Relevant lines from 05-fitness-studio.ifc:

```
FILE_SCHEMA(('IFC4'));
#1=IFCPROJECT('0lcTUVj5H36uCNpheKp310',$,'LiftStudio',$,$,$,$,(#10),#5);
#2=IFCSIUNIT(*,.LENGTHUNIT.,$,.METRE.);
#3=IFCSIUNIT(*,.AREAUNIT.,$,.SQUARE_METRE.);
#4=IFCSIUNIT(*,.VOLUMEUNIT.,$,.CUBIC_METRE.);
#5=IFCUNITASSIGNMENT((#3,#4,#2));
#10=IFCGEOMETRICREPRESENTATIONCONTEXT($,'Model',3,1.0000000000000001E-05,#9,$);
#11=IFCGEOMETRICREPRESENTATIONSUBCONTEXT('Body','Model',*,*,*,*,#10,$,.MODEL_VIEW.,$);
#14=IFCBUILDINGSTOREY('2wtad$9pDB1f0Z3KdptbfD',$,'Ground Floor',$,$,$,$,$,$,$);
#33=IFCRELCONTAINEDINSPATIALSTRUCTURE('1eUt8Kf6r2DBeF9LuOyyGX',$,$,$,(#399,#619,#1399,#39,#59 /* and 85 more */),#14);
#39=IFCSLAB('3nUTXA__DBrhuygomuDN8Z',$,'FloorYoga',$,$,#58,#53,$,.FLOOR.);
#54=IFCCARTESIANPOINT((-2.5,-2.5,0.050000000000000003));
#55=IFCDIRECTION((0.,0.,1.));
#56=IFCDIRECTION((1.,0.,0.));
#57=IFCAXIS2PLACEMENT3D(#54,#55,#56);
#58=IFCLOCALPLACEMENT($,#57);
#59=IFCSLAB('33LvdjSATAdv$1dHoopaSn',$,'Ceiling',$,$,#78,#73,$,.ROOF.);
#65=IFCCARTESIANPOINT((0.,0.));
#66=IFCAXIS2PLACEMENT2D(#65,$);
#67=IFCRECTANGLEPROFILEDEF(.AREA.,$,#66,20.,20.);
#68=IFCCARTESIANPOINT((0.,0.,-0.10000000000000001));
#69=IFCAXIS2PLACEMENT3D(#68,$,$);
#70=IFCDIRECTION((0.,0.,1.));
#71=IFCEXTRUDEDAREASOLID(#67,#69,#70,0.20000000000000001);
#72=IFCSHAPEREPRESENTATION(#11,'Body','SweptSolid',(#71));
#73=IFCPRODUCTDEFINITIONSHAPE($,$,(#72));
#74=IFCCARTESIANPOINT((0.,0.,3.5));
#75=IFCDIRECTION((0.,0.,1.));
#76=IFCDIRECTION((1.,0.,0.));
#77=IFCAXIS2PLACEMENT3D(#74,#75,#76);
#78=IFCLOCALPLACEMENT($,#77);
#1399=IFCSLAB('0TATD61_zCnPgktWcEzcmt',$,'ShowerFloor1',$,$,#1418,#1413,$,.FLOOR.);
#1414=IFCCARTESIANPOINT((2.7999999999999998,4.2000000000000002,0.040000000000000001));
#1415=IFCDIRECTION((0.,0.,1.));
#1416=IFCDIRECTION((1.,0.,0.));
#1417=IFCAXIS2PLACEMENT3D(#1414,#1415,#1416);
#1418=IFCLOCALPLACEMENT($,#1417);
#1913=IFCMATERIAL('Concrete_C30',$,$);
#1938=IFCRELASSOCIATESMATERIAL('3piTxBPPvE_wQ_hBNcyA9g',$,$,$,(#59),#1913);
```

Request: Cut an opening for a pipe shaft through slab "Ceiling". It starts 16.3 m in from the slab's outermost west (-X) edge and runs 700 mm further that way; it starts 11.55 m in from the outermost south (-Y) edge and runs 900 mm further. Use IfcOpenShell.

```python
import numpy as np
import ifcopenshell
import ifcopenshell.api.feature
import ifcopenshell.api.geometry
import ifcopenshell.api.root
import ifcopenshell.geom
import ifcopenshell.util.placement
import ifcopenshell.util.representation
import ifcopenshell.util.shape
import ifcopenshell.util.unit

model = ifcopenshell.open("05-fitness-studio.ifc")
unit_scale = ifcopenshell.util.unit.calculate_unit_scale(model)
settings = ifcopenshell.geom.settings()


def volume(element):
    """Net volume in cubic metres, openings subtracted."""
    shape = ifcopenshell.geom.create_shape(settings, element)
    return ifcopenshell.util.shape.get_volume(shape.geometry)


slab = model.by_guid("33LvdjSATAdv$1dHoopaSn")
before = volume(slab)

# Extent in the slab's own axes, in metres. The edges named are its -X and -Y sides.
slab_shape = ifcopenshell.geom.create_shape(settings, slab)
vertices = ifcopenshell.util.shape.get_vertices(slab_shape.geometry)
x_min, y_min, bottom = vertices.min(axis=0)
top = vertices[:, 2].max()

opening = ifcopenshell.api.root.create_entity(model, ifc_class="IfcOpeningElement", name="Pipe shaft opening", predefined_type="OPENING")
context = ifcopenshell.util.representation.get_context(model, "Model", "Body", "MODEL_VIEW")
width, depth = 0.7, 0.9
outline = [(0.0, 0.0), (width, 0.0), (width, depth), (0.0, depth), (0.0, 0.0)]
# Overshoot both faces by 50 mm so the cut is clean.
shape = ifcopenshell.api.geometry.add_slab_representation(
    model, context=context, depth=top - bottom + 0.1, polyline=outline
)
ifcopenshell.api.geometry.assign_representation(model, product=opening, representation=shape)

matrix = ifcopenshell.util.placement.get_local_placement(slab.ObjectPlacement)
matrix[:, 3] = matrix @ np.append(np.array([x_min + 16.3, y_min + 11.55, bottom - 0.05]) / unit_scale, 1.0)
ifcopenshell.api.geometry.edit_object_placement(model, product=opening, matrix=matrix, is_si=False)
ifcopenshell.api.feature.add_feature(model, feature=opening, element=slab)

after = volume(slab)

print(f"slab volume {before:.3f} -> {after:.3f} m3")

model.write("05-fitness-studio_updated.ifc")
```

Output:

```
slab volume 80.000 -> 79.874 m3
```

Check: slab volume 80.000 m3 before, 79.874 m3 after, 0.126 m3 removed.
